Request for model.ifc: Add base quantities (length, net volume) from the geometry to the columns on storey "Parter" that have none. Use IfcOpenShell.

First a look at what the model holds.

```python
import ifcopenshell
import ifcopenshell.util.element
import ifcopenshell.util.unit

model = ifcopenshell.open("model.ifc")
print(model.schema)
for unit_type in ("LENGTHUNIT", "AREAUNIT", "VOLUMEUNIT"):
    print(unit_type, ifcopenshell.util.unit.calculate_unit_scale(model, unit_type))
storey = next(s for s in model.by_type("IfcBuildingStorey") if s.Name == "Parter")
columns = [e for e in ifcopenshell.util.element.get_decomposition(storey) if e.is_a("IfcColumn")]
for e in sorted(columns, key=lambda e: e.id()):
    print(e.id(), e.is_a(), e.Name, list(ifcopenshell.util.element.get_psets(e, qtos_only=True)), sep=" | ")
```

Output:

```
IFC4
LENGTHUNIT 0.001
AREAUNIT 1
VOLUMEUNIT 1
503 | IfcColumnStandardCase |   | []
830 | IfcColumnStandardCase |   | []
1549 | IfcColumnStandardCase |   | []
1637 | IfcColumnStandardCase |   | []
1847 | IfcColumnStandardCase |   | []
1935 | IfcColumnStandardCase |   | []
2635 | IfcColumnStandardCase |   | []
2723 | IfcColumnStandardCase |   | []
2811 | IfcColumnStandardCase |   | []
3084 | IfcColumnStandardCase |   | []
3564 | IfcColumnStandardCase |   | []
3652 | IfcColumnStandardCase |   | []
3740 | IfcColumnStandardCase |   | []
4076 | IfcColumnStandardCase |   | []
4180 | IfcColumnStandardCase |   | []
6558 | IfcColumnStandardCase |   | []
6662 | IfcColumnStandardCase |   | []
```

```python
import ifcopenshell
import ifcopenshell.api.pset
import ifcopenshell.geom
import ifcopenshell.util.element
import ifcopenshell.util.shape
import ifcopenshell.util.unit

model = ifcopenshell.open("model.ifc")
unit_scale = ifcopenshell.util.unit.calculate_unit_scale(model)
volume_scale = ifcopenshell.util.unit.calculate_unit_scale(model, "VOLUMEUNIT")
settings = ifcopenshell.geom.settings()

storey = next(s for s in model.by_type("IfcBuildingStorey") if s.Name == "Parter")
columns = [e for e in ifcopenshell.util.element.get_decomposition(storey) if e.is_a("IfcColumn")]

for e in sorted(columns, key=lambda e: e.id()):
    if ifcopenshell.util.element.get_psets(e, qtos_only=True, should_inherit=False):
        continue
    # Geometry comes back in metres, in the element's own axes.
    shape = ifcopenshell.geom.create_shape(settings, e)
    values = {
        "Length": ifcopenshell.util.shape.get_z(shape.geometry) / unit_scale,
        "NetVolume": ifcopenshell.util.shape.get_volume(shape.geometry) / volume_scale,
    }
    qto = ifcopenshell.api.pset.add_qto(model, product=e, name="Qto_ColumnBaseQuantities")
    ifcopenshell.api.pset.edit_qto(model, qto=qto, properties=values)
    print(e.id(), {k: round(v, 3) for k, v in values.items()})

model.write("model_v2.ifc")
```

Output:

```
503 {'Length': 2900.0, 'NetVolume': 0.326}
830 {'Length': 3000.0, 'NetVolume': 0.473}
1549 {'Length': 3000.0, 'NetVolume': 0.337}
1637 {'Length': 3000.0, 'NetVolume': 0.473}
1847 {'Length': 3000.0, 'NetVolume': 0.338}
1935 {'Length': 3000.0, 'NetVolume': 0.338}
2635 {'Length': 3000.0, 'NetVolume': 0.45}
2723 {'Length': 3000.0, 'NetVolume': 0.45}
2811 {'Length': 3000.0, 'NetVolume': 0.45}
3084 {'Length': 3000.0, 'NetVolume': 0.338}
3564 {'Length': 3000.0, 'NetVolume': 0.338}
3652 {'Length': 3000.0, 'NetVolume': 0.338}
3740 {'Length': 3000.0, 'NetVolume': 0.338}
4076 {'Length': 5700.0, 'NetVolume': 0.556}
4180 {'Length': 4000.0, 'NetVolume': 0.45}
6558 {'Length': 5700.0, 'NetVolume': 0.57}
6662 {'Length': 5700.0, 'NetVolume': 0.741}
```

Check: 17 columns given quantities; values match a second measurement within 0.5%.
